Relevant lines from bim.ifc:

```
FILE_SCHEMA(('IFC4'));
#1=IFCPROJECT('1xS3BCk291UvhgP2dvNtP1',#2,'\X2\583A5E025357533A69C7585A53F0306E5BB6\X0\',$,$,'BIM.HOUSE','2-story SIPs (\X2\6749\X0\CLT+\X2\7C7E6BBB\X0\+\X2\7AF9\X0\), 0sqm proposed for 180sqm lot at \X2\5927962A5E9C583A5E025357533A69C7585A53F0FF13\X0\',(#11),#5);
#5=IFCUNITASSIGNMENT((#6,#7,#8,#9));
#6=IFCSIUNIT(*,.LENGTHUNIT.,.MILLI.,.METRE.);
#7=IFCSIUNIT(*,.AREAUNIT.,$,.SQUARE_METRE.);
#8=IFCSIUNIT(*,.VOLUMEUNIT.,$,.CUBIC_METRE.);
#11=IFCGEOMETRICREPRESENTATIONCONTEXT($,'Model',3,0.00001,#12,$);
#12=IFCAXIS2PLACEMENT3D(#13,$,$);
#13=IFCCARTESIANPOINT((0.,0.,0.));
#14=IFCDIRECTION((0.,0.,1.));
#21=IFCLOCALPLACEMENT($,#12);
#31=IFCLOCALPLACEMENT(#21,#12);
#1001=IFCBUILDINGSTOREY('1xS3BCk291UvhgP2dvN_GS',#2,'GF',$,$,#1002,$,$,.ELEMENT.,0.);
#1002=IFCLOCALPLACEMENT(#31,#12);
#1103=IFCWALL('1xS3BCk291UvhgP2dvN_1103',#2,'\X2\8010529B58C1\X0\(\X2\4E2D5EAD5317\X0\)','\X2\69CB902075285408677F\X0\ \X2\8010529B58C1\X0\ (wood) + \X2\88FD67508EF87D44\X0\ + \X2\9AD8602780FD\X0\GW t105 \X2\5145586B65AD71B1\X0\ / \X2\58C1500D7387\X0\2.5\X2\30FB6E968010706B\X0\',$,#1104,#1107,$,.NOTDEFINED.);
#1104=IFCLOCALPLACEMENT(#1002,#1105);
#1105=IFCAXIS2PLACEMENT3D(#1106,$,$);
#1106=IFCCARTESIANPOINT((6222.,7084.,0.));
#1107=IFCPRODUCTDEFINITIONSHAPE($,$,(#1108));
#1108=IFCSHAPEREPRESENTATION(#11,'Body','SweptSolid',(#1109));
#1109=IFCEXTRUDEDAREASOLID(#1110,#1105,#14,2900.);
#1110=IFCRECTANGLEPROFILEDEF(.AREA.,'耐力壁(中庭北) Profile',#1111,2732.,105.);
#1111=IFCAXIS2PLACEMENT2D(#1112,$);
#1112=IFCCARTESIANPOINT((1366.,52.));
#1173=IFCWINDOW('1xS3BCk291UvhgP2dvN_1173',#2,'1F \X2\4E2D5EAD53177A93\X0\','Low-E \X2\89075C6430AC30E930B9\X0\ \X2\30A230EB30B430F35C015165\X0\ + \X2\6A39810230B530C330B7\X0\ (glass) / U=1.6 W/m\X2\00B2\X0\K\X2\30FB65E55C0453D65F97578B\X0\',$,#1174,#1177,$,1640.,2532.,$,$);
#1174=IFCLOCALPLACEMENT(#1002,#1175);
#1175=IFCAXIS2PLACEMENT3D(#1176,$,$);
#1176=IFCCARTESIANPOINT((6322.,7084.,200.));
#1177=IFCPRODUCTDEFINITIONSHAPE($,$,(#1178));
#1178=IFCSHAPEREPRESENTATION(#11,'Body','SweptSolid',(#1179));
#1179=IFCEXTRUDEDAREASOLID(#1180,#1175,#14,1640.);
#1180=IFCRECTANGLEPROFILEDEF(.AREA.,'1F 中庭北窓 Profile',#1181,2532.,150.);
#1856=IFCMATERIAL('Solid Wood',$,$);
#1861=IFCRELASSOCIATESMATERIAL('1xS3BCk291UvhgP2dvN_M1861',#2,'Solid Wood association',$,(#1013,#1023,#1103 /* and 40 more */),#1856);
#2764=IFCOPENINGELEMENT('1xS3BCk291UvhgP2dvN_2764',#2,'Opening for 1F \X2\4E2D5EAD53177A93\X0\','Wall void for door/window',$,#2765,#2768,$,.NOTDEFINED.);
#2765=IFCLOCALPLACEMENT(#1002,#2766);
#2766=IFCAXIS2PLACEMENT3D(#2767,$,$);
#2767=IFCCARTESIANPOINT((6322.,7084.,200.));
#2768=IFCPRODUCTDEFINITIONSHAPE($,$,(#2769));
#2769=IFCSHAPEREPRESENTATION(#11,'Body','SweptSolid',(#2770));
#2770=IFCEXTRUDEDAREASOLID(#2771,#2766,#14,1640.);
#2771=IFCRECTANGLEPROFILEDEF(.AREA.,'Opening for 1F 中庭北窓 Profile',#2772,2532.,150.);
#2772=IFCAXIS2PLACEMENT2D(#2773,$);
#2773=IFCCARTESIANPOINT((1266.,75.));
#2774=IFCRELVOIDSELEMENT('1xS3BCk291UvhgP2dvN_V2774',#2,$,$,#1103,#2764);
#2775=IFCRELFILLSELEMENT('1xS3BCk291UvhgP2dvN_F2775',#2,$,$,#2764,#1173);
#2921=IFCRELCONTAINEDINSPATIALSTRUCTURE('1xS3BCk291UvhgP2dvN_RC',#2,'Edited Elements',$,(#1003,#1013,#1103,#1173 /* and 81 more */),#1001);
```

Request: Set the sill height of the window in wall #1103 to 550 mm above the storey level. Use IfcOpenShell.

```python
import numpy as np
import ifcopenshell
import ifcopenshell.api.geometry
import ifcopenshell.geom
import ifcopenshell.util.element
import ifcopenshell.util.placement
import ifcopenshell.util.shape
import ifcopenshell.util.unit

model = ifcopenshell.open("bim.ifc")
unit_scale = ifcopenshell.util.unit.calculate_unit_scale(model)

window = model.by_id(1173)
opening = window.FillsVoids[0].RelatingOpeningElement
storey = ifcopenshell.util.element.get_container(window, ifc_class="IfcBuildingStorey")
level = ifcopenshell.util.placement.get_local_placement(storey.ObjectPlacement)[2, 3]

# The opening's origin need not be at the sill, so measure its lowest point.
shape = ifcopenshell.geom.create_shape(ifcopenshell.geom.settings(), opening)
bottom = ifcopenshell.util.shape.get_shape_bottom_elevation(shape, shape.geometry) / unit_scale
dz = level + 0.55 / unit_scale - bottom

shift = np.array([0.0, 0.0, dz])
# The window is not placed relative to its opening, so move both.
for product in (opening, window):
    matrix = ifcopenshell.util.placement.get_local_placement(product.ObjectPlacement)
    matrix[:3, 3] += shift
    ifcopenshell.api.geometry.edit_object_placement(model, product=product, matrix=matrix, is_si=False)

print(f"moved by {dz * unit_scale:+.3f} m")

model.write("bim_updated.ifc")
```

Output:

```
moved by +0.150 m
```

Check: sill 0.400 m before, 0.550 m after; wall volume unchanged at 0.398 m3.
